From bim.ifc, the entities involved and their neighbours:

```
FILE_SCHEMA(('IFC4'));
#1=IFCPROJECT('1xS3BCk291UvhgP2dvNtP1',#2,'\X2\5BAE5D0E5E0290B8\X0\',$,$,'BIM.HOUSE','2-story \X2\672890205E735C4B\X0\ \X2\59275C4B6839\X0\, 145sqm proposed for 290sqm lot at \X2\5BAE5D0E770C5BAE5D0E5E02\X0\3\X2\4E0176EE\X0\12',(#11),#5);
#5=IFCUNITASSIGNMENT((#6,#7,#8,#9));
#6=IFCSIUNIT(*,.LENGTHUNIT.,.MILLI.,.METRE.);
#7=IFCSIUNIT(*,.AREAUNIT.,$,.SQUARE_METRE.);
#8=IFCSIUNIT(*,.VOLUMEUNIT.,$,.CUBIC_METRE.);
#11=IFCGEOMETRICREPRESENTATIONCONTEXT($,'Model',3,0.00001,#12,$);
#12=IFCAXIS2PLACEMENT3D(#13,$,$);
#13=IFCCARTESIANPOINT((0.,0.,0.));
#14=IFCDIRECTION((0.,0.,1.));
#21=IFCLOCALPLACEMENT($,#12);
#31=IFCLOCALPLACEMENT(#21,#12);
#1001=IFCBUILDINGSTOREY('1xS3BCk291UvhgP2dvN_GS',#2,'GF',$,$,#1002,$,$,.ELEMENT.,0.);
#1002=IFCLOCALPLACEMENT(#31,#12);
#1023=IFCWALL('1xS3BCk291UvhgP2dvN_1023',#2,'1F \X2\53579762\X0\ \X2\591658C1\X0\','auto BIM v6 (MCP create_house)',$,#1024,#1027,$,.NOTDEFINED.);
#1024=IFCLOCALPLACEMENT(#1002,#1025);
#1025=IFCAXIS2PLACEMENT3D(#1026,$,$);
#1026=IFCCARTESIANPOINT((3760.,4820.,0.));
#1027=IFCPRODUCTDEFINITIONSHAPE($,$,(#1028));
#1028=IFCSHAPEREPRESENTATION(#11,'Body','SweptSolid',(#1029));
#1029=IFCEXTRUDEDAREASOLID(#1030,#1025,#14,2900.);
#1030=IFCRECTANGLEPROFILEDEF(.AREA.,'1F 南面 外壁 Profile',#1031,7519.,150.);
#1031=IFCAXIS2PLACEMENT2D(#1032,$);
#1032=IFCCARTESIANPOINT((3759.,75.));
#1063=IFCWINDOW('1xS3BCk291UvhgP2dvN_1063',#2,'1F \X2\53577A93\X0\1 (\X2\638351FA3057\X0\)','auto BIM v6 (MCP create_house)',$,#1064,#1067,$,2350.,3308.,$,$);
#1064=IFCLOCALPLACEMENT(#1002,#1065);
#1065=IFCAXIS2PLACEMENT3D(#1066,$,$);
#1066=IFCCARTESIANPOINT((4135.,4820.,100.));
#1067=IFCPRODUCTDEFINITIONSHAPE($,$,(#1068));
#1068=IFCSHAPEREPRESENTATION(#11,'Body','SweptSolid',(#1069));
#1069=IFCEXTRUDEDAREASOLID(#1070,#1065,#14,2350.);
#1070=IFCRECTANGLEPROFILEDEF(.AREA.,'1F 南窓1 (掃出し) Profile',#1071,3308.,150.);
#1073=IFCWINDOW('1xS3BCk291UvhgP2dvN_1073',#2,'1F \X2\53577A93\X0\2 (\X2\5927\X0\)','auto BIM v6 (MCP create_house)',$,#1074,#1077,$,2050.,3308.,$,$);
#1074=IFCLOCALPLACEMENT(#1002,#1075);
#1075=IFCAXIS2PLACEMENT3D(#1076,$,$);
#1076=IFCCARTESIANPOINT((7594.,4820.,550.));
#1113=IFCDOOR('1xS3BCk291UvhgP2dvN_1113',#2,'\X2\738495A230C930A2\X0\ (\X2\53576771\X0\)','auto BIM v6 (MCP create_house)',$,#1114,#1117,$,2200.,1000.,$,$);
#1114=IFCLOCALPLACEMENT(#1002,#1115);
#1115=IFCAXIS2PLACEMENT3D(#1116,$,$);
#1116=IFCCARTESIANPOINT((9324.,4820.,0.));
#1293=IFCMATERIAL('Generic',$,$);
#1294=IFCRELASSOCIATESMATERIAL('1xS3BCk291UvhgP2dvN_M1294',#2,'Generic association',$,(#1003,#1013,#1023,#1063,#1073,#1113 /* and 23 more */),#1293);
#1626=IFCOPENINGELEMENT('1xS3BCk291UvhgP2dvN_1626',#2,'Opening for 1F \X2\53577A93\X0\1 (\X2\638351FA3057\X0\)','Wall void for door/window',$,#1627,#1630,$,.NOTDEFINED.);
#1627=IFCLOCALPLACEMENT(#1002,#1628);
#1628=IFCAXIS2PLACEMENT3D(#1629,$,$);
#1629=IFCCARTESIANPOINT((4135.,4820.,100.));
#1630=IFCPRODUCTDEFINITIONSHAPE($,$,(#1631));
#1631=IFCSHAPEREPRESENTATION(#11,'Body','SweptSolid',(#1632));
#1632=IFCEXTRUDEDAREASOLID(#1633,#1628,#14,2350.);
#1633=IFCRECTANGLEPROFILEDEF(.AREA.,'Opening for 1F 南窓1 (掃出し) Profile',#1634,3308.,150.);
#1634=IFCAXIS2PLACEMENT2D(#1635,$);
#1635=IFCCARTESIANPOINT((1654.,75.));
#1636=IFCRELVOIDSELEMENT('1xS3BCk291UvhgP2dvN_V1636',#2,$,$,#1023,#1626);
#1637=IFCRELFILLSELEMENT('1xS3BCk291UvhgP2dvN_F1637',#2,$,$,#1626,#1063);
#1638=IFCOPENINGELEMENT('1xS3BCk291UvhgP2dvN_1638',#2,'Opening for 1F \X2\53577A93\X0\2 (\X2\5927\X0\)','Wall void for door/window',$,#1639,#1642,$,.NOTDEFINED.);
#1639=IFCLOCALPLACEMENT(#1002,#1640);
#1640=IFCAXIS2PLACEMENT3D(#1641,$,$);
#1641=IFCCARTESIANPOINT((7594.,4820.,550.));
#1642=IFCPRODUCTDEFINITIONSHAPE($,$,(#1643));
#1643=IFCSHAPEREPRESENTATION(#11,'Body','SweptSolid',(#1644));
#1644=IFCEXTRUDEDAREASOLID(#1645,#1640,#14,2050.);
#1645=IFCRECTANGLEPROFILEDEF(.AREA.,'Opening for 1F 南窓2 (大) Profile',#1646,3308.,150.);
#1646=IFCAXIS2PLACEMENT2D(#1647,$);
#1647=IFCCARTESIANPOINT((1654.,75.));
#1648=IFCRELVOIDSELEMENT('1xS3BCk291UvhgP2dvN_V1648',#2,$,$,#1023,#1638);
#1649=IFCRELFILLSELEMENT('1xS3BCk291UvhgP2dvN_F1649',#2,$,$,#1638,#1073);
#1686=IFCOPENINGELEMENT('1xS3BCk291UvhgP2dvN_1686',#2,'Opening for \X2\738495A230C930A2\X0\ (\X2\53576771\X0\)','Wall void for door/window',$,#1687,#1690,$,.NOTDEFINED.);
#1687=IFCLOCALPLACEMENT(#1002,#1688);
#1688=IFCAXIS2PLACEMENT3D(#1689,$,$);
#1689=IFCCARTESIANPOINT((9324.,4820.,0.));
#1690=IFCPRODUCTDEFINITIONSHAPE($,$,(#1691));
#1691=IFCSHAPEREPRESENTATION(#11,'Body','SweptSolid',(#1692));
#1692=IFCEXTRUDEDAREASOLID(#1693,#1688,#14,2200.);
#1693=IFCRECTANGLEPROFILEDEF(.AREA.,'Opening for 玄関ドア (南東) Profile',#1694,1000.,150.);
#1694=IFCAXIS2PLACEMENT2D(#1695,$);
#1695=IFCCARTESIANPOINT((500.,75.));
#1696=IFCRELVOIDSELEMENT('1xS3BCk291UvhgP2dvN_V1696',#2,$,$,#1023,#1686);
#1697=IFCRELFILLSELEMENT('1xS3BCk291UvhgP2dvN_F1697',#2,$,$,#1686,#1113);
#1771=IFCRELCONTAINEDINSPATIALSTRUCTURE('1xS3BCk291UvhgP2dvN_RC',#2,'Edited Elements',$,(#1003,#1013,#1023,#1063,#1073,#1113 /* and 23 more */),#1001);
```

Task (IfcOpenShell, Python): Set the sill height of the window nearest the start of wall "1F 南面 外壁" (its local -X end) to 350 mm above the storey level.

```python
import numpy as np
import ifcopenshell
import ifcopenshell.api.geometry
import ifcopenshell.geom
import ifcopenshell.util.element
import ifcopenshell.util.placement
import ifcopenshell.util.shape
import ifcopenshell.util.unit

model = ifcopenshell.open("bim.ifc")
unit_scale = ifcopenshell.util.unit.calculate_unit_scale(model)

window = model.by_guid("1xS3BCk291UvhgP2dvN_1063")
opening = window.FillsVoids[0].RelatingOpeningElement
storey = ifcopenshell.util.element.get_container(window, ifc_class="IfcBuildingStorey")
level = ifcopenshell.util.placement.get_local_placement(storey.ObjectPlacement)[2, 3]

# The opening's origin need not be at the sill, so measure its lowest point.
shape = ifcopenshell.geom.create_shape(ifcopenshell.geom.settings(), opening)
bottom = ifcopenshell.util.shape.get_shape_bottom_elevation(shape, shape.geometry) / unit_scale
dz = level + 0.35 / unit_scale - bottom

shift = np.array([0.0, 0.0, dz])
# The window is not placed relative to its opening, so move both.
for product in (opening, window):
    matrix = ifcopenshell.util.placement.get_local_placement(product.ObjectPlacement)
    matrix[:3, 3] += shift
    ifcopenshell.api.geometry.edit_object_placement(model, product=product, matrix=matrix, is_si=False)

print(f"moved by {dz * unit_scale:+.3f} m")

model.write("bim_v2.ifc")
```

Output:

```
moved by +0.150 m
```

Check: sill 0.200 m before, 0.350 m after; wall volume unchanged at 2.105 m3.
